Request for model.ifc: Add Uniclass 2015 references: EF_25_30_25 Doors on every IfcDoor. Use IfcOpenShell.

First a look at what the model holds.

```python
import ifcopenshell

model = ifcopenshell.open("model.ifc")
print(model.schema)
print("classifications:", [c.Name for c in model.by_type("IfcClassification")])
for ifc_class in ("IfcDoor", "IfcRoof", "IfcStair", "IfcWall", "IfcWindow"):
    print(ifc_class, len(model.by_type(ifc_class)))
```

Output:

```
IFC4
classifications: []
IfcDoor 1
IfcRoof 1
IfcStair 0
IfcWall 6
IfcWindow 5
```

```python
import ifcopenshell
import ifcopenshell.api.classification

model = ifcopenshell.open("model.ifc")

system = ifcopenshell.api.classification.add_classification(model, classification="Uniclass 2015")

codes = {
    "IfcDoor": ("EF_25_30_25", "Doors"),
}
for ifc_class, (code, name) in codes.items():
    products = model.by_type(ifc_class)
    ifcopenshell.api.classification.add_reference(
        model, products=products, classification=system, identification=code, name=name
    )
    print(code, len(products))

model.write("model_edited.ifc")
```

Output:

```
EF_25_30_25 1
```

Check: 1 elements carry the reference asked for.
